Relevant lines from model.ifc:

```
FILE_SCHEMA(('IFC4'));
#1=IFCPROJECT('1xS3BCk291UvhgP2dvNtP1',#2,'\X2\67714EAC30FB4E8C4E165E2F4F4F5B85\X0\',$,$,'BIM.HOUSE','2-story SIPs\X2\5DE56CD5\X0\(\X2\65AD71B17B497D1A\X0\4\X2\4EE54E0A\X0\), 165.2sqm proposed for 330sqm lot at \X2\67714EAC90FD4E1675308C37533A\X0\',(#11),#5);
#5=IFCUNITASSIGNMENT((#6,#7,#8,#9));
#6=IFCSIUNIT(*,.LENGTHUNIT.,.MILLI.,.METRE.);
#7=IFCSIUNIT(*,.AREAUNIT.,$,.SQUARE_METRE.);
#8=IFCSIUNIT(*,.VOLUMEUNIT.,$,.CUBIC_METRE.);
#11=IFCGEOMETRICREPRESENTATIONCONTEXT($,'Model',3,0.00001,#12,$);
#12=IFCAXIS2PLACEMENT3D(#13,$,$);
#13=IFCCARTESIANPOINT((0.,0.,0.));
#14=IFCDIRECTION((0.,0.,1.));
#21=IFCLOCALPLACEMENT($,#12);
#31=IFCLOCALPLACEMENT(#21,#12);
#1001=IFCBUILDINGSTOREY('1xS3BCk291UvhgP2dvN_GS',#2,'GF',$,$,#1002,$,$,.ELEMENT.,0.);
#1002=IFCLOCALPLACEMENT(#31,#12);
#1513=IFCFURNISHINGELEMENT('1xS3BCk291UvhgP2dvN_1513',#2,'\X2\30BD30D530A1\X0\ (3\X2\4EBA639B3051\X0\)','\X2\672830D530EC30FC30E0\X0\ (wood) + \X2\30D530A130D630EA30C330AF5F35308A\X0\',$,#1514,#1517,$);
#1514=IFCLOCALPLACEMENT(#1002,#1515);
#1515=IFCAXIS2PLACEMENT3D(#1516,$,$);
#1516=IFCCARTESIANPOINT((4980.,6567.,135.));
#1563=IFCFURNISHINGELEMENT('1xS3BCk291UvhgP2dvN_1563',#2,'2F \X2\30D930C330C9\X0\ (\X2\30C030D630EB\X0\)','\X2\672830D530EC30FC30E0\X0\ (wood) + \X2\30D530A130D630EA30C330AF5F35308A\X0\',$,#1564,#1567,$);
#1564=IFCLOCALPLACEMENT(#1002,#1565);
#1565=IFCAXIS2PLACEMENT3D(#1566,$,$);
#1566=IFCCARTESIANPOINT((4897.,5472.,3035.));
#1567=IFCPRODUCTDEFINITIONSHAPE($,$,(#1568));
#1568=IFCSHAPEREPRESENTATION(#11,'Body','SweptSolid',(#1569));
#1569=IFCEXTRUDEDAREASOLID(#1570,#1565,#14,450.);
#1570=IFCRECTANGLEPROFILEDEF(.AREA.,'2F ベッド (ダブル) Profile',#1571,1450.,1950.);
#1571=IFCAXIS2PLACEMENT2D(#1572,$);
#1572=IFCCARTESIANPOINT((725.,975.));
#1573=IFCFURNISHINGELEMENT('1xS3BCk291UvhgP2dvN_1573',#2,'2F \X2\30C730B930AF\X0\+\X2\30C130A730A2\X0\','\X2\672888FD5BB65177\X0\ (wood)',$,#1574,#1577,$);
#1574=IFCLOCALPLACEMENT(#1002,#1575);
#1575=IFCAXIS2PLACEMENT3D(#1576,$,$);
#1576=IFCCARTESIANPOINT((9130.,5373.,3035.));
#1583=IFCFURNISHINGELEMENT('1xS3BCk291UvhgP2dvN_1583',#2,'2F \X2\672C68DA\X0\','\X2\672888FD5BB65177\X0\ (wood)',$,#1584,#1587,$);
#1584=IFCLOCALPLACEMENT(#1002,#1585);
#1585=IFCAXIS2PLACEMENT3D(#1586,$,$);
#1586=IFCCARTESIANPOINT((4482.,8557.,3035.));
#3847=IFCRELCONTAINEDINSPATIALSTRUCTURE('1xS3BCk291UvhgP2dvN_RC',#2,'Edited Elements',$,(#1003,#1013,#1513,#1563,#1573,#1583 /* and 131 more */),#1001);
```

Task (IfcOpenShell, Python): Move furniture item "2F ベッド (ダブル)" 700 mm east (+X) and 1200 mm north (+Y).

```python
import ifcopenshell
import ifcopenshell.api.geometry
import ifcopenshell.util.placement
import ifcopenshell.util.unit

model = ifcopenshell.open("model.ifc")
unit_scale = ifcopenshell.util.unit.calculate_unit_scale(model)

item = model.by_guid("1xS3BCk291UvhgP2dvN_1563")
matrix = ifcopenshell.util.placement.get_local_placement(item.ObjectPlacement)
matrix[0, 3] += 0.7 / unit_scale
matrix[1, 3] += 1.2 / unit_scale
ifcopenshell.api.geometry.edit_object_placement(model, product=item, matrix=matrix, is_si=False)

print(ifcopenshell.util.placement.get_local_placement(item.ObjectPlacement).round(3) + 0.0)

model.write("model-out.ifc")
```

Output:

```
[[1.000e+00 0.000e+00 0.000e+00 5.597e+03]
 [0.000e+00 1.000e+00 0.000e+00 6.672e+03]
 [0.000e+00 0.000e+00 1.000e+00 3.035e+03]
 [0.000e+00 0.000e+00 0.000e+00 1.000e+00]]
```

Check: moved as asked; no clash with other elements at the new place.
